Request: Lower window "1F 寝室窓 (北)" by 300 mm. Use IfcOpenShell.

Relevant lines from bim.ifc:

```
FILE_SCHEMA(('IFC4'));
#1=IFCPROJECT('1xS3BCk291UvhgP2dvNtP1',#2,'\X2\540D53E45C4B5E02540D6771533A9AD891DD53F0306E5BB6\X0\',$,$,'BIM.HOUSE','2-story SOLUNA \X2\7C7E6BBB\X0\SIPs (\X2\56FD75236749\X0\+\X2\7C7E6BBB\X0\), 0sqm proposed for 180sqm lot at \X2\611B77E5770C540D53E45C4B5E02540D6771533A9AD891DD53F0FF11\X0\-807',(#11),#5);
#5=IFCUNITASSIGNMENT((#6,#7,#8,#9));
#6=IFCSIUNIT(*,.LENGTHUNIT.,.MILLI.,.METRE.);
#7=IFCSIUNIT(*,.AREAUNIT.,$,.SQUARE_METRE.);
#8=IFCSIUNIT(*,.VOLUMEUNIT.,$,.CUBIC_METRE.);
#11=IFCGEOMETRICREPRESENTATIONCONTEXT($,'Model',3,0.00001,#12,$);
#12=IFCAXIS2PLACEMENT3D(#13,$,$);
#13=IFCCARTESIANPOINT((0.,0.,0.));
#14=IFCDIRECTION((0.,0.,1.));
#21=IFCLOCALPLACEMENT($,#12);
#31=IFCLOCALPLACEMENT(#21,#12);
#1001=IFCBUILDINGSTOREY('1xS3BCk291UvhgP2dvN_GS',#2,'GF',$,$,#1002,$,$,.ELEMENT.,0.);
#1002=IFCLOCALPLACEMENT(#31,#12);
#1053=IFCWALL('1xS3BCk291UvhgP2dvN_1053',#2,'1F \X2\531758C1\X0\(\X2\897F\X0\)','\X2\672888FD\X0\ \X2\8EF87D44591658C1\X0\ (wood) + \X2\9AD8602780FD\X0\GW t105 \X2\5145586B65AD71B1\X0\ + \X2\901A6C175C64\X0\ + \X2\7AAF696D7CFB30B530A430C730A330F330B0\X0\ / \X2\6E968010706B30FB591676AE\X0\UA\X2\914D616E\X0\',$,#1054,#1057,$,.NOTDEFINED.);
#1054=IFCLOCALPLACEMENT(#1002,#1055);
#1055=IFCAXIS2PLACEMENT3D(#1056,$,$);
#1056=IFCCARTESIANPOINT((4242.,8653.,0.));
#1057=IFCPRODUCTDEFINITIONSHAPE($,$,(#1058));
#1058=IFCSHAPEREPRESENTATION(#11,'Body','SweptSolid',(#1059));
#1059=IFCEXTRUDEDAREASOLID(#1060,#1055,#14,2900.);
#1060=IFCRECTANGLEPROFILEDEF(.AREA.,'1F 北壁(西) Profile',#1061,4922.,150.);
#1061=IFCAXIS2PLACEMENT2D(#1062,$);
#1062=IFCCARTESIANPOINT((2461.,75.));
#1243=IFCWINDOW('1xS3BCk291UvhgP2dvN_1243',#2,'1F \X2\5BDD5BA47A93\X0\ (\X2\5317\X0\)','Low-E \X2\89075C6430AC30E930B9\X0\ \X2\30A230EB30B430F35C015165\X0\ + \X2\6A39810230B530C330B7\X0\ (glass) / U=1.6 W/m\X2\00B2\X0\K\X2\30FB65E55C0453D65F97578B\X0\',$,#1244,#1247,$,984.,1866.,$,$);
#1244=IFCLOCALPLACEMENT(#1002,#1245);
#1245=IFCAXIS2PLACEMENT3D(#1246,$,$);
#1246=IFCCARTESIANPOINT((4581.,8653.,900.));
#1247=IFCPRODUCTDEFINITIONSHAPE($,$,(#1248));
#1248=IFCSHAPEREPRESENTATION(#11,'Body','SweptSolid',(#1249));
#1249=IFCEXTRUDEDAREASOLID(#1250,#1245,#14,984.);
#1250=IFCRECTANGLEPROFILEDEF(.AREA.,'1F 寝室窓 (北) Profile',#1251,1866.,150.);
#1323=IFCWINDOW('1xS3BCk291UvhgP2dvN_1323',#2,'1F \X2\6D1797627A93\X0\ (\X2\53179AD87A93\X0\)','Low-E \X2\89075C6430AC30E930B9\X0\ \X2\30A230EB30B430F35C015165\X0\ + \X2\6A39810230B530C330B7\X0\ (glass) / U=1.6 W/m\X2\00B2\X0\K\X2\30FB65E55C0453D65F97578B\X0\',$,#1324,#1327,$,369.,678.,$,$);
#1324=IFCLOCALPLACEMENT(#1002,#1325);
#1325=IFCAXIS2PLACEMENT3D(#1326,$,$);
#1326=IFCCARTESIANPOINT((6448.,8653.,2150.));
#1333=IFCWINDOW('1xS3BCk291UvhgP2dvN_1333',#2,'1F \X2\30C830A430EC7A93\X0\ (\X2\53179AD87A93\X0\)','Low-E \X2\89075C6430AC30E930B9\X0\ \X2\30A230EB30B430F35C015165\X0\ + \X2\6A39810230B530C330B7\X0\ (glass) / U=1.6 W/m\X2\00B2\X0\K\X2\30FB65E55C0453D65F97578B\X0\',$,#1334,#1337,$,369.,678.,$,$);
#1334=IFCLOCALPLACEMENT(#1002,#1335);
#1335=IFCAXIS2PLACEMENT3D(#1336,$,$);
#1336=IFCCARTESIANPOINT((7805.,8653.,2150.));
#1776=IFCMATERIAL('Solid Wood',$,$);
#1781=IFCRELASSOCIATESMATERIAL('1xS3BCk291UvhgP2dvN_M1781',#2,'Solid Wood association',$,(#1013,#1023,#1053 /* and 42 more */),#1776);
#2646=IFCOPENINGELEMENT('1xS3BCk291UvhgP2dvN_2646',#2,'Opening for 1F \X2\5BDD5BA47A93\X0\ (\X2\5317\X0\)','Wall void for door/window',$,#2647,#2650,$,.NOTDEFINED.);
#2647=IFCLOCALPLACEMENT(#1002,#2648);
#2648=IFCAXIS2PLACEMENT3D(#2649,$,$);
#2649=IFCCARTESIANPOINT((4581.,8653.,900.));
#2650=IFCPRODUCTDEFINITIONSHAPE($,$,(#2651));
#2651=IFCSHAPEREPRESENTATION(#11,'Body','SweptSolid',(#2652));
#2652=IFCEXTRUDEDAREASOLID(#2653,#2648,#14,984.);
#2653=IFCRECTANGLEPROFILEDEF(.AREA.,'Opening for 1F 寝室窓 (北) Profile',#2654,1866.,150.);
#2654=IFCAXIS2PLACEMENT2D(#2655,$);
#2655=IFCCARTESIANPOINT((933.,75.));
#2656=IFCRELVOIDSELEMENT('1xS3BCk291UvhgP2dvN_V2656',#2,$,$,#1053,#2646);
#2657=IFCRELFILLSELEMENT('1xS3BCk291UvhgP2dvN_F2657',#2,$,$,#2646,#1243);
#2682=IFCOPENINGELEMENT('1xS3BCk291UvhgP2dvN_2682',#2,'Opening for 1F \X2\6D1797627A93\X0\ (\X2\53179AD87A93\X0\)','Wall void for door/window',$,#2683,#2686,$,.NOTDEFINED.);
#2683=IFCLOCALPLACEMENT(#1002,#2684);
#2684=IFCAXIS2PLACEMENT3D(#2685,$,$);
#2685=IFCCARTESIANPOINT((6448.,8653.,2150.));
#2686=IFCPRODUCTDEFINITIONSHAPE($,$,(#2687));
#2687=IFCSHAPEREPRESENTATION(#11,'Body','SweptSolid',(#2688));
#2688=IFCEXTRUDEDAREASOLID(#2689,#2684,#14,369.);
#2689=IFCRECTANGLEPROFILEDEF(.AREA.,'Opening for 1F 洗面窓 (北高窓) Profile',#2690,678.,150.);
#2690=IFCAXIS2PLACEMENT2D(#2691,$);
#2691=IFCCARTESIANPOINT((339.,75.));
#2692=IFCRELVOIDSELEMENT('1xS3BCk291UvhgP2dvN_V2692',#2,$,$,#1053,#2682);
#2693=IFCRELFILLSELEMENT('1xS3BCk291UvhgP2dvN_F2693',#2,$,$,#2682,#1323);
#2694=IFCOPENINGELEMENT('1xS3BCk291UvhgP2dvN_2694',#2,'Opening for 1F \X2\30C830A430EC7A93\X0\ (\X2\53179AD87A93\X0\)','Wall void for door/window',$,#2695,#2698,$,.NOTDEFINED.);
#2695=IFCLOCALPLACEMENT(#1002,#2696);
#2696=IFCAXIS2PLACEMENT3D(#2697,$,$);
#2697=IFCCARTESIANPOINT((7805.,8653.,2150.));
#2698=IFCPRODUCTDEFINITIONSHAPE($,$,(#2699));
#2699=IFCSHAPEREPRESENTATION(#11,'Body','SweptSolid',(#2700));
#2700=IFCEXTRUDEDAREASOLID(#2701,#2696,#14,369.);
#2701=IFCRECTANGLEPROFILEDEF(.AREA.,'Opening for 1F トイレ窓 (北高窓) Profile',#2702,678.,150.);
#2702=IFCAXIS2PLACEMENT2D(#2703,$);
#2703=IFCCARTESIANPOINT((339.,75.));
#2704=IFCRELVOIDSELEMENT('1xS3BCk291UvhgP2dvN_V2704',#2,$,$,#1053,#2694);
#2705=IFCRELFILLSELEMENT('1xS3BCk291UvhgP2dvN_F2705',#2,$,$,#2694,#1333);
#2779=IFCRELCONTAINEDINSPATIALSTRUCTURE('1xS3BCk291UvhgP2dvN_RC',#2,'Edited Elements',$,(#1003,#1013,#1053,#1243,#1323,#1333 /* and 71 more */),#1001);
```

```python
import numpy as np
import ifcopenshell
import ifcopenshell.api.geometry
import ifcopenshell.util.placement
import ifcopenshell.util.unit

model = ifcopenshell.open("bim.ifc")
unit_scale = ifcopenshell.util.unit.calculate_unit_scale(model)

window = model.by_id(1243)
opening = window.FillsVoids[0].RelatingOpeningElement
dz = -300.0

shift = np.array([0.0, 0.0, dz])
# The window is not placed relative to its opening, so move both.
for product in (opening, window):
    matrix = ifcopenshell.util.placement.get_local_placement(product.ObjectPlacement)
    matrix[:3, 3] += shift
    ifcopenshell.api.geometry.edit_object_placement(model, product=product, matrix=matrix, is_si=False)

print(f"moved by {dz * unit_scale:+.3f} m")

model.write("bim-out.ifc")
```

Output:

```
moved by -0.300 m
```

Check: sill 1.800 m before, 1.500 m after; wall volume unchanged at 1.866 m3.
